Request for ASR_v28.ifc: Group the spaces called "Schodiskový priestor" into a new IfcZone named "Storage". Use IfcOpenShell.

First a look at what the model holds.

```python
import ifcopenshell

model = ifcopenshell.open("ASR_v28.ifc")
print(model.schema)
seen = {}
for space in model.by_type("IfcSpace"):
    seen[space.LongName] = seen.get(space.LongName, 0) + 1
for name, count in sorted(seen.items(), key=str):
    print(count, "x", name)
print("zones:", [z.Name for z in model.by_type("IfcZone")][:20])
```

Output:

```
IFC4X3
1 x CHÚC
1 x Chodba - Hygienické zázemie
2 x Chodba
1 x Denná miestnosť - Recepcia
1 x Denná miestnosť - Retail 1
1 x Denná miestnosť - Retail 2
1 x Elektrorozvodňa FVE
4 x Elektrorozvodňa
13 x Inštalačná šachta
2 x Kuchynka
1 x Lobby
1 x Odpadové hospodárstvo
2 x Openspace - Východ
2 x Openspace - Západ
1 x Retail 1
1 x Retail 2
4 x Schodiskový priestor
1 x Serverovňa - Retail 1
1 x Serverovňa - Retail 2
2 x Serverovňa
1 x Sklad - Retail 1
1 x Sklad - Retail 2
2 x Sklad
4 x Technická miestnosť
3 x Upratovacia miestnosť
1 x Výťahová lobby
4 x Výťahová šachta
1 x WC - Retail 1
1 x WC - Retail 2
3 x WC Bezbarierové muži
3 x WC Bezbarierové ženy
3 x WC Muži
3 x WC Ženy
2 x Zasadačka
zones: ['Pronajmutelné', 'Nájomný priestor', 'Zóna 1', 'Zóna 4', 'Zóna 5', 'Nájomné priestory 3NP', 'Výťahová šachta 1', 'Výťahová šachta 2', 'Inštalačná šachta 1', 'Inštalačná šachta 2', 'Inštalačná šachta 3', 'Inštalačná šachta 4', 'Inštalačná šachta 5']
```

```python
import ifcopenshell
import ifcopenshell.api.group
import ifcopenshell.api.root

model = ifcopenshell.open("ASR_v28.ifc")

names = {"Schodiskový priestor"}
spaces = [s for s in model.by_type("IfcSpace") if s.LongName in names]

zone = ifcopenshell.api.root.create_entity(model, ifc_class="IfcZone", name="Storage")
ifcopenshell.api.group.assign_group(model, products=spaces, group=zone)
print(len(spaces), "spaces in", zone.Name)

model.write("ASR_v28_v2.ifc")
```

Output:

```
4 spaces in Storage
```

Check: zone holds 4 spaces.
